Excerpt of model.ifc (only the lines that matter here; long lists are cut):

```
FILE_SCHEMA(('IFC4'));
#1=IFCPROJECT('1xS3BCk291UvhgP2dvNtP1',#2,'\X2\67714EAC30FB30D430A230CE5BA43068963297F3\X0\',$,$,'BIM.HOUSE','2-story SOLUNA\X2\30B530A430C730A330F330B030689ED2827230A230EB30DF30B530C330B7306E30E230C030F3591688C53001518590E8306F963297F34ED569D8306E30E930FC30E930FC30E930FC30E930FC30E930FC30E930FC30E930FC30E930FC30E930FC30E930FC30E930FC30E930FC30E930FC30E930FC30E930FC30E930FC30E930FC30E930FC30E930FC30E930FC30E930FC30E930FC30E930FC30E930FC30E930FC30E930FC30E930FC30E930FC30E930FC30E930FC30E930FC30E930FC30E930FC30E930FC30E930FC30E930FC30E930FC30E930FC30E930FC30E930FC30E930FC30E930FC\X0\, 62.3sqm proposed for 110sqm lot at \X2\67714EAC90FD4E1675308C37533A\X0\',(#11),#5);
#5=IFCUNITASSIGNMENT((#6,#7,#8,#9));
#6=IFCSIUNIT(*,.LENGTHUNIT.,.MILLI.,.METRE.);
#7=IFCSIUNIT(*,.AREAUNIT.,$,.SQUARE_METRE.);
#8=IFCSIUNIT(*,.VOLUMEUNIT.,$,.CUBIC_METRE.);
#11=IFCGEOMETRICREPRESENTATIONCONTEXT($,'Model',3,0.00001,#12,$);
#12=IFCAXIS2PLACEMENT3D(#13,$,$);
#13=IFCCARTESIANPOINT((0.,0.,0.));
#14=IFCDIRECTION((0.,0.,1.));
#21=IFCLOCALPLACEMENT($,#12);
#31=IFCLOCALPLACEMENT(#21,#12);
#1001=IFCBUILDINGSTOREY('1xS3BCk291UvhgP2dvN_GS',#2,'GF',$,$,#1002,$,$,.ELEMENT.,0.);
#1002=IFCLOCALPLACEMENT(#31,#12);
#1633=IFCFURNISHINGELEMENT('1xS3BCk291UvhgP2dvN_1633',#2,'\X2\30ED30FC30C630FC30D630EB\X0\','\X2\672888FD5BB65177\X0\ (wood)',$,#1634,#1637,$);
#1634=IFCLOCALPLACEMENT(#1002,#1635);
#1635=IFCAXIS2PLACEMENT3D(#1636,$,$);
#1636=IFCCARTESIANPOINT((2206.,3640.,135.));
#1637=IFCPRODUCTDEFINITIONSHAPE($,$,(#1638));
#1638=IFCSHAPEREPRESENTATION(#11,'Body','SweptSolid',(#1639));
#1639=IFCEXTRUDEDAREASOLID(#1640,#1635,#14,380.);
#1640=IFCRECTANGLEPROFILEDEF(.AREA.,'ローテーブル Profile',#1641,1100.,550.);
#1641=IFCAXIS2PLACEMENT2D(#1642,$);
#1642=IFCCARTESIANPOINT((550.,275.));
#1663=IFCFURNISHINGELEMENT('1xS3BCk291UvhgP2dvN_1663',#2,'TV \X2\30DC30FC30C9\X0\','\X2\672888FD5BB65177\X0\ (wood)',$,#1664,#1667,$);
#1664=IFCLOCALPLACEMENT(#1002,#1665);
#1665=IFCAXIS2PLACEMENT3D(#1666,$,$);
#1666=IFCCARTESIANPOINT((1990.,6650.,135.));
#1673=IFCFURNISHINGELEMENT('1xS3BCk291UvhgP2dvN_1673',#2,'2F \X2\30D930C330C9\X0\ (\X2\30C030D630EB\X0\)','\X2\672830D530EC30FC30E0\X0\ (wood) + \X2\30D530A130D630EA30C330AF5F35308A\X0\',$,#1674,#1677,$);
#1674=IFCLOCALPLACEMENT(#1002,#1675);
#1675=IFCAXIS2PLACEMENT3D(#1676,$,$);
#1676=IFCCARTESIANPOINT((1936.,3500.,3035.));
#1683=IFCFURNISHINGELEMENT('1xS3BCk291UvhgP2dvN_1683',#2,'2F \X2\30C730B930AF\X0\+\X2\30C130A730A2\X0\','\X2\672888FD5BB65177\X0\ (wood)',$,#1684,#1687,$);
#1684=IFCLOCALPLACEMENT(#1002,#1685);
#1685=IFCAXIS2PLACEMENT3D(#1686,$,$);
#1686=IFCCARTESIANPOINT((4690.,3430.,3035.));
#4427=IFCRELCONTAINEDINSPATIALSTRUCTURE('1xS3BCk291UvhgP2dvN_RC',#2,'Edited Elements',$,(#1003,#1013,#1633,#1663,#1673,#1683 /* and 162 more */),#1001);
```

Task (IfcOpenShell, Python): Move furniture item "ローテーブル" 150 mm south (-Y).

```python
import ifcopenshell
import ifcopenshell.api.geometry
import ifcopenshell.util.placement
import ifcopenshell.util.unit

model = ifcopenshell.open("model.ifc")
unit_scale = ifcopenshell.util.unit.calculate_unit_scale(model)

item = model.by_guid("1xS3BCk291UvhgP2dvN_1633")
matrix = ifcopenshell.util.placement.get_local_placement(item.ObjectPlacement)
matrix[1, 3] -= 0.15 / unit_scale
ifcopenshell.api.geometry.edit_object_placement(model, product=item, matrix=matrix, is_si=False)

print(ifcopenshell.util.placement.get_local_placement(item.ObjectPlacement).round(3) + 0.0)

model.write("model_edited.ifc")
```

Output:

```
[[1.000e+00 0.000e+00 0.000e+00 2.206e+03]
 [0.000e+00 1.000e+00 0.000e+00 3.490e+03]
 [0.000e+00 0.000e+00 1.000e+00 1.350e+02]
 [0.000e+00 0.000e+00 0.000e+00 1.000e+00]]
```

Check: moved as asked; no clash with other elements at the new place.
